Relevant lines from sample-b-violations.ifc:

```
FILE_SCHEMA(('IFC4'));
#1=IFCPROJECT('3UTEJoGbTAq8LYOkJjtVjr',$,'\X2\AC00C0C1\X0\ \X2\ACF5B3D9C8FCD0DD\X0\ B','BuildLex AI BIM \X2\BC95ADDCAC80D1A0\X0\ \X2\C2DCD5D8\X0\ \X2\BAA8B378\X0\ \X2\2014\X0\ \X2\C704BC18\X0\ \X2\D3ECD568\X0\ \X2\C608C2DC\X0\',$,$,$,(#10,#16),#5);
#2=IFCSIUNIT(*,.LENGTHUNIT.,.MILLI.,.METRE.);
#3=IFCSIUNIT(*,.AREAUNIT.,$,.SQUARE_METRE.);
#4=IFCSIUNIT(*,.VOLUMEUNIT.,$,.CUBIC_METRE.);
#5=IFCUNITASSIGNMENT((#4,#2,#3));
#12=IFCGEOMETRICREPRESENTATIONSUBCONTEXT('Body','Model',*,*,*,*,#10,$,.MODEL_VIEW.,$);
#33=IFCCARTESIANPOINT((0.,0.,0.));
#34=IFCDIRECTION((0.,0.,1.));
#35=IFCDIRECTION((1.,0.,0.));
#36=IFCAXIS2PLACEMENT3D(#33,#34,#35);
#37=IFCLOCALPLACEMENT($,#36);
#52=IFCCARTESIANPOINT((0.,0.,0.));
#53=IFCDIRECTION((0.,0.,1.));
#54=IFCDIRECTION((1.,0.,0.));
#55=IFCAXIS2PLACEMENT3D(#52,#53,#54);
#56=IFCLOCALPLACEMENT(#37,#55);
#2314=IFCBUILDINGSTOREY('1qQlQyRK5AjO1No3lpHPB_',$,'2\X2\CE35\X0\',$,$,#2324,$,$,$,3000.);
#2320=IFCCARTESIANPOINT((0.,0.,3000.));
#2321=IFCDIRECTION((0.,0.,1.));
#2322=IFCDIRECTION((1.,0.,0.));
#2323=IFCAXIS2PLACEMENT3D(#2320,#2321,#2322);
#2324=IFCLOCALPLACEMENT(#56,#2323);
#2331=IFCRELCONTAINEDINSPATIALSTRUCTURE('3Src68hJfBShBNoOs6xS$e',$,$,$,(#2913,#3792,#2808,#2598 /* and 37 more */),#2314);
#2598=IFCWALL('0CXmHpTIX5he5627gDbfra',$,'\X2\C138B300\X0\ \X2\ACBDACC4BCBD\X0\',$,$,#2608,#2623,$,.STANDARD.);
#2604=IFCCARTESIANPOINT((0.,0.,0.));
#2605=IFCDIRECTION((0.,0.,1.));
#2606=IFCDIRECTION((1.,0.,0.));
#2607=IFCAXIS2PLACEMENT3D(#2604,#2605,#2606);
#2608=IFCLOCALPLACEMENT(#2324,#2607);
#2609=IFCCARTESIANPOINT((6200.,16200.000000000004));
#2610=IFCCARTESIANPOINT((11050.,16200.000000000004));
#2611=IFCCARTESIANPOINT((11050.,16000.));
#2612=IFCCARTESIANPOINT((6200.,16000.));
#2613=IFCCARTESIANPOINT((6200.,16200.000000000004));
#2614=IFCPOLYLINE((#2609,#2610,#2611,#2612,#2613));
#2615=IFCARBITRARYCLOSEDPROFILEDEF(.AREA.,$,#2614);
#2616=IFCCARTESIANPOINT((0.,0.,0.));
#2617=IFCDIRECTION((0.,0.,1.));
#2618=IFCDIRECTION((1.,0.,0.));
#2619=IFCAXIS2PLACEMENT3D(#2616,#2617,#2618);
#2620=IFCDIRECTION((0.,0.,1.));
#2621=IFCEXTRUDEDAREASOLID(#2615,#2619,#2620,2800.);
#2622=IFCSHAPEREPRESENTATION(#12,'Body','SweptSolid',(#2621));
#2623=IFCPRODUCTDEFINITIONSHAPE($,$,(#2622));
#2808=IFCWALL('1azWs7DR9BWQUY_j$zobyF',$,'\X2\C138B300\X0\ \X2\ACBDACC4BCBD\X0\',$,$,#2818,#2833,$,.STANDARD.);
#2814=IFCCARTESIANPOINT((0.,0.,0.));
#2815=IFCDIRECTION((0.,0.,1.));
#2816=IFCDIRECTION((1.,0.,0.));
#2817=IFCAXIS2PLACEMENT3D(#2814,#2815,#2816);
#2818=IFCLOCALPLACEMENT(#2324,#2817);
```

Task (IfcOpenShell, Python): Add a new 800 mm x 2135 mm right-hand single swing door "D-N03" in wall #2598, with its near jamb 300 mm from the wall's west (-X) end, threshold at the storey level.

```python
import numpy as np
import ifcopenshell
import ifcopenshell.api.feature
import ifcopenshell.api.geometry
import ifcopenshell.api.root
import ifcopenshell.api.spatial
import ifcopenshell.geom
import ifcopenshell.util.element
import ifcopenshell.util.placement
import ifcopenshell.util.representation
import ifcopenshell.util.shape
import ifcopenshell.util.unit

model = ifcopenshell.open("sample-b-violations.ifc")
unit_scale = ifcopenshell.util.unit.calculate_unit_scale(model)
settings = ifcopenshell.geom.settings()


def volume(element):
    """Net volume in cubic metres, openings subtracted."""
    shape = ifcopenshell.geom.create_shape(settings, element)
    return ifcopenshell.util.shape.get_volume(shape.geometry)


wall = model.by_guid("0CXmHpTIX5he5627gDbfra")
storey = ifcopenshell.util.element.get_container(wall, ifc_class="IfcBuildingStorey")
context = ifcopenshell.util.representation.get_context(model, "Model", "Body", "MODEL_VIEW")
before = volume(wall)

width, height, from_end, sill = 0.8, 2.135, 0.3, 0.0  # metres

# The wall runs along its own X axis, and the end named is its -X end.
wall_shape = ifcopenshell.geom.create_shape(settings, wall)
x, y, z = ifcopenshell.util.shape.get_vertices(wall_shape.geometry).T
start = x.min() + from_end
face, thickness = float(y.min()), float(y.max() - y.min())
wall_matrix = ifcopenshell.util.placement.get_local_placement(wall.ObjectPlacement)
level = ifcopenshell.util.placement.get_local_placement(storey.ObjectPlacement)[2, 3]


def in_wall(x, y):
    """Placement at x, y metres in the wall's axes, at sill height."""
    matrix = wall_matrix.copy()
    matrix[:, 3] = wall_matrix @ np.array([x / unit_scale, y / unit_scale, 0.0, 1.0])
    matrix[2, 3] = level + sill / unit_scale
    return matrix


# Opening: a box that overshoots both wall faces by 50 mm.
opening = ifcopenshell.api.root.create_entity(model, ifc_class="IfcOpeningElement", predefined_type="OPENING")
box = ifcopenshell.api.geometry.add_wall_representation(
    model, context=context, length=width, height=height, thickness=thickness + 0.1
)
ifcopenshell.api.geometry.assign_representation(model, product=opening, representation=box)
ifcopenshell.api.geometry.edit_object_placement(model, product=opening, matrix=in_wall(start, face - 0.05), is_si=False)
ifcopenshell.api.feature.add_feature(model, feature=opening, element=wall)

door = ifcopenshell.api.root.create_entity(model, ifc_class="IfcDoor", name="D-N03", predefined_type="DOOR")
door.OverallWidth, door.OverallHeight = width / unit_scale, height / unit_scale
door.OperationType = "SINGLE_SWING_RIGHT"
body = ifcopenshell.api.geometry.add_door_representation(
    model,
    context=context,
    overall_width=door.OverallWidth,
    overall_height=door.OverallHeight,
    operation_type="SINGLE_SWING_RIGHT",
    lining_properties={"LiningDepth": thickness / unit_scale, "ThresholdDepth": thickness / unit_scale},
)
ifcopenshell.api.geometry.assign_representation(model, product=door, representation=body)
ifcopenshell.api.spatial.assign_container(model, products=[door], relating_structure=storey)
ifcopenshell.api.feature.add_filling(model, opening=opening, element=door)

# The lining spans the wall, so the door starts at the wall face.
ifcopenshell.api.geometry.edit_object_placement(model, product=door, matrix=in_wall(start, face), is_si=False)

after = volume(wall)

print(f"wall volume {before:.3f} -> {after:.3f} m3")

model.write("sample-b-violations_rev.ifc")
```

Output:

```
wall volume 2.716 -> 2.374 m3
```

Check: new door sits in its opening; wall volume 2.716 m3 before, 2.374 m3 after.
